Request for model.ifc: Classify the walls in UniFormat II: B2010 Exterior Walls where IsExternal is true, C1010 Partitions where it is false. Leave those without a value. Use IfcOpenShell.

First a look at what the model holds.

```python
import ifcopenshell
import ifcopenshell.util.element

model = ifcopenshell.open("model.ifc")
print(model.schema)
print("classifications:", [c.Name for c in model.by_type("IfcClassification")])
values = [ifcopenshell.util.element.get_pset(e, "Pset_WallCommon", "IsExternal") for e in model.by_type("IfcWall")]
for value in (True, False, None):
    print("IsExternal", value, values.count(value))
```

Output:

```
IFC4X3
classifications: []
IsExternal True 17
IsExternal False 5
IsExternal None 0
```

```python
import ifcopenshell
import ifcopenshell.api.classification
import ifcopenshell.util.element

model = ifcopenshell.open("model.ifc")

system = ifcopenshell.api.classification.add_classification(model, classification="UniFormat II")

walls = model.by_type("IfcWall")
external = {e: ifcopenshell.util.element.get_pset(e, "Pset_WallCommon", "IsExternal") for e in walls}
for flag, code, name in ((True, "B2010", "Exterior Walls"), (False, "C1010", "Partitions")):
    products = [e for e in walls if external[e] is flag]
    ifcopenshell.api.classification.add_reference(
        model, products=products, classification=system, identification=code, name=name
    )
    print(code, len(products))

model.write("model_rev.ifc")
```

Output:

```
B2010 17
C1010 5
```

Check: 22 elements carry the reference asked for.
